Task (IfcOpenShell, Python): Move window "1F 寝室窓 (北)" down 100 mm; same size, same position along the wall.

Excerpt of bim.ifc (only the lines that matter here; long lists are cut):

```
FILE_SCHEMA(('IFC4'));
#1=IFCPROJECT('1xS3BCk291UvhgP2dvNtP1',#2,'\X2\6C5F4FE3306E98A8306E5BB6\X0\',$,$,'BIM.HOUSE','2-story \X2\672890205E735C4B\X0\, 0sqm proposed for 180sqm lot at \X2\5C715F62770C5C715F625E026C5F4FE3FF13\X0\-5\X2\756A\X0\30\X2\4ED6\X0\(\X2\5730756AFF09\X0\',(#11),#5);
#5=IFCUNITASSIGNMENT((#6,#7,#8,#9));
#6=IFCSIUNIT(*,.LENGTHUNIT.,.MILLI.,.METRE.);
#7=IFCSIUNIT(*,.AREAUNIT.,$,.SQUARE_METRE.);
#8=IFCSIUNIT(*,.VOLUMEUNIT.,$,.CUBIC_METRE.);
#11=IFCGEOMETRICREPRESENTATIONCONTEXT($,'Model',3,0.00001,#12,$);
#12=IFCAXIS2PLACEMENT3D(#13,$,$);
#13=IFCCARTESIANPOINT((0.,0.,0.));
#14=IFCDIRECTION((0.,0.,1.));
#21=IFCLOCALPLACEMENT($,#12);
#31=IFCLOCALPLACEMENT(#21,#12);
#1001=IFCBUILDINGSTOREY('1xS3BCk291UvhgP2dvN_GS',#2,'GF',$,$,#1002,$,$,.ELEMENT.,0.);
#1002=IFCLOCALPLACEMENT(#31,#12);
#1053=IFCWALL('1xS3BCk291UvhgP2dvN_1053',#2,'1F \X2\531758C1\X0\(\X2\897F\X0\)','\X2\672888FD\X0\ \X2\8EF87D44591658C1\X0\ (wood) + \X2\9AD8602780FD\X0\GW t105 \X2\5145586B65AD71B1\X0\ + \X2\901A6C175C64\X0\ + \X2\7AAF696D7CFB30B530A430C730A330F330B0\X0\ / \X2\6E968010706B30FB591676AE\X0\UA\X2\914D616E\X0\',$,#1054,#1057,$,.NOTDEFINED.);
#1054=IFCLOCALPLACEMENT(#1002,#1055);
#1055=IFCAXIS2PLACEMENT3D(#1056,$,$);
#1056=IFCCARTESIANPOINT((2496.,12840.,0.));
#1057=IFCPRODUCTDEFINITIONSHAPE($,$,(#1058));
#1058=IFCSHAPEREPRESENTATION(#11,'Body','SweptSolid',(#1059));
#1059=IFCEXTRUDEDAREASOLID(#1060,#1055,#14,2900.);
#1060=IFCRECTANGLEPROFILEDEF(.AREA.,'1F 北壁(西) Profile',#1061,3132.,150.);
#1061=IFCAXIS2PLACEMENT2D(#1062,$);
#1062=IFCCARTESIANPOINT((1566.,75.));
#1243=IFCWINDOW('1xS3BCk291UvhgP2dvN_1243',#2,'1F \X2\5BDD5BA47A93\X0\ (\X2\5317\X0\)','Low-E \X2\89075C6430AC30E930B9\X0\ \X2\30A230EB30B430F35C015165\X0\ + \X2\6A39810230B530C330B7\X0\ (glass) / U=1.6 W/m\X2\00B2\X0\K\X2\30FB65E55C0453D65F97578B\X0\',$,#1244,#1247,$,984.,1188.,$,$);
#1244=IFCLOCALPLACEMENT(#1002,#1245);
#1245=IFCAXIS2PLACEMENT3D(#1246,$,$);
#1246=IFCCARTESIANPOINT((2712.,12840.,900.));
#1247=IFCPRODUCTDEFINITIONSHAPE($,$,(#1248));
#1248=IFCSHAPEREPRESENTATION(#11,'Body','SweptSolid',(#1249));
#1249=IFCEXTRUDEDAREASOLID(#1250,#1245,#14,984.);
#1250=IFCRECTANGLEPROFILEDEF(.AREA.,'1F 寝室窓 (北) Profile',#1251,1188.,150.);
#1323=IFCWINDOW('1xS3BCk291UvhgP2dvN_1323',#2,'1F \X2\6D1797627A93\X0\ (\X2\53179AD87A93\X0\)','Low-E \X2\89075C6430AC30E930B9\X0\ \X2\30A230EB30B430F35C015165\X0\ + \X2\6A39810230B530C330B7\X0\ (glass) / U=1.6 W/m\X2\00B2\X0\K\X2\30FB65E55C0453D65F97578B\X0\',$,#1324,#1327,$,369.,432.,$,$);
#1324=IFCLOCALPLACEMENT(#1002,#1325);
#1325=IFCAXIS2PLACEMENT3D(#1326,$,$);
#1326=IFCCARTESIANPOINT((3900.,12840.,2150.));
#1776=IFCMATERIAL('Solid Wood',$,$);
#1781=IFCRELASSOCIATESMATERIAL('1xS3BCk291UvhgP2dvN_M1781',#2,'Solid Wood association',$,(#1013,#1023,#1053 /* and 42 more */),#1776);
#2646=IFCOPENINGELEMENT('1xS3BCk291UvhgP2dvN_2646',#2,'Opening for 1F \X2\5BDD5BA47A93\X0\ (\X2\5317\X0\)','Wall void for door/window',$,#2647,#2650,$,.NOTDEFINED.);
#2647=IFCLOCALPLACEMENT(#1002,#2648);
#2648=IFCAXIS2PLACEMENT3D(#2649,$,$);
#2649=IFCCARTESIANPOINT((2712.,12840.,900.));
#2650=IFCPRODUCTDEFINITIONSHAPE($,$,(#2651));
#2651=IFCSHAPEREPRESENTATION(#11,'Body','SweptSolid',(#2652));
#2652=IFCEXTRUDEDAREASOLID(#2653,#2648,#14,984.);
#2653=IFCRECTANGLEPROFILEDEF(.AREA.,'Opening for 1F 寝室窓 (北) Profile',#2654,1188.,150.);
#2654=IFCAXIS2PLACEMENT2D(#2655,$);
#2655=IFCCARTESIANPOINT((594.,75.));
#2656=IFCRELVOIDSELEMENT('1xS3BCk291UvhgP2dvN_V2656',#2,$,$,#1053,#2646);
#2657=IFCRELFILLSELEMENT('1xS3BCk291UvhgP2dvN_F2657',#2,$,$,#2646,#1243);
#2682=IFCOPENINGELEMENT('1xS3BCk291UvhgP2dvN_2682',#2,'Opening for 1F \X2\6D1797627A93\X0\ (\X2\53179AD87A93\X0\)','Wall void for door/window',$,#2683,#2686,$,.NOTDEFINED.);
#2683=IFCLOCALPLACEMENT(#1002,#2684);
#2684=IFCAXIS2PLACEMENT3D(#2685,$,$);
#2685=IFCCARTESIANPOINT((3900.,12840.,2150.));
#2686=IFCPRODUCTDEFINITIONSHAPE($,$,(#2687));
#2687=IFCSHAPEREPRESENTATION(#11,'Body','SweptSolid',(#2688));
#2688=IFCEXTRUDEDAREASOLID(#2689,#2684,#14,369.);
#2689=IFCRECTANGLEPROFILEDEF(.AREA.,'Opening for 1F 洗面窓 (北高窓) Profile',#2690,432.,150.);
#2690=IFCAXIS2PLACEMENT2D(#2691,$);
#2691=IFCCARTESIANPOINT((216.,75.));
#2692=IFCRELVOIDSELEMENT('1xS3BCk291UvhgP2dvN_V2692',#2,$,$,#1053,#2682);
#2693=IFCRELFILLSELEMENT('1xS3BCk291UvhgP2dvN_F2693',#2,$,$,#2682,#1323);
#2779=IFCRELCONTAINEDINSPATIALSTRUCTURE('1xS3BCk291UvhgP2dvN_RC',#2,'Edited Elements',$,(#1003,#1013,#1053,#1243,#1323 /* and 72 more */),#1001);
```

```python
import numpy as np
import ifcopenshell
import ifcopenshell.api.geometry
import ifcopenshell.util.placement
import ifcopenshell.util.unit

model = ifcopenshell.open("bim.ifc")
unit_scale = ifcopenshell.util.unit.calculate_unit_scale(model)

window = model.by_guid("1xS3BCk291UvhgP2dvN_1243")
opening = window.FillsVoids[0].RelatingOpeningElement
dz = -0.1 / unit_scale

shift = np.array([0.0, 0.0, dz])
# The window is not placed relative to its opening, so move both.
for product in (opening, window):
    matrix = ifcopenshell.util.placement.get_local_placement(product.ObjectPlacement)
    matrix[:3, 3] += shift
    ifcopenshell.api.geometry.edit_object_placement(model, product=product, matrix=matrix, is_si=False)

print(f"moved by {dz * unit_scale:+.3f} m")

model.write("bim-out.ifc")
```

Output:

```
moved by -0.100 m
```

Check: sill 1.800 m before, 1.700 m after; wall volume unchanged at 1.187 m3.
